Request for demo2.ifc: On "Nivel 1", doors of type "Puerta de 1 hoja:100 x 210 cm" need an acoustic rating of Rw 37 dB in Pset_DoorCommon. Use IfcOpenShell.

First a look at what the model holds.

```python
import ifcopenshell
import ifcopenshell.util.element

model = ifcopenshell.open("demo2.ifc")
print(model.schema)
storey = next(s for s in model.by_type("IfcBuildingStorey") if s.Name == "Nivel 1")
doors = [e for e in ifcopenshell.util.element.get_decomposition(storey) if e.is_a("IfcDoor")]
seen = {}
for e in doors:
    element_type = ifcopenshell.util.element.get_type(e)
    key = (element_type.Name if element_type != e and element_type else None, ifcopenshell.util.element.get_pset(e, "Pset_DoorCommon", "AcousticRating"))
    seen[key] = seen.get(key, 0) + 1
for (name, value), count in sorted(seen.items(), key=str):
    print(count, "x", name, "|", value)
```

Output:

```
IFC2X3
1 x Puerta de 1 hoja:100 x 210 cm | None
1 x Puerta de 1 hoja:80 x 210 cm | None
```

```python
import ifcopenshell
import ifcopenshell.api.pset
import ifcopenshell.util.element

model = ifcopenshell.open("demo2.ifc")

storey = next(s for s in model.by_type("IfcBuildingStorey") if s.Name == "Nivel 1")
doors = [e for e in ifcopenshell.util.element.get_decomposition(storey) if e.is_a("IfcDoor")]

count = 0
for e in doors:
    element_type = ifcopenshell.util.element.get_type(e)
    if element_type in (None, e) or element_type.Name != "Puerta de 1 hoja:100 x 210 cm":
        continue
    # add_pset returns the element's existing set when there is one.
    pset = ifcopenshell.api.pset.add_pset(model, product=e, name="Pset_DoorCommon")
    ifcopenshell.api.pset.edit_pset(model, pset=pset, properties={"AcousticRating": "Rw 37 dB"})
    count += 1

print(count, "doors updated")

model.write("demo2_v2.ifc")
```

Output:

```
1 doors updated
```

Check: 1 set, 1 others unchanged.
